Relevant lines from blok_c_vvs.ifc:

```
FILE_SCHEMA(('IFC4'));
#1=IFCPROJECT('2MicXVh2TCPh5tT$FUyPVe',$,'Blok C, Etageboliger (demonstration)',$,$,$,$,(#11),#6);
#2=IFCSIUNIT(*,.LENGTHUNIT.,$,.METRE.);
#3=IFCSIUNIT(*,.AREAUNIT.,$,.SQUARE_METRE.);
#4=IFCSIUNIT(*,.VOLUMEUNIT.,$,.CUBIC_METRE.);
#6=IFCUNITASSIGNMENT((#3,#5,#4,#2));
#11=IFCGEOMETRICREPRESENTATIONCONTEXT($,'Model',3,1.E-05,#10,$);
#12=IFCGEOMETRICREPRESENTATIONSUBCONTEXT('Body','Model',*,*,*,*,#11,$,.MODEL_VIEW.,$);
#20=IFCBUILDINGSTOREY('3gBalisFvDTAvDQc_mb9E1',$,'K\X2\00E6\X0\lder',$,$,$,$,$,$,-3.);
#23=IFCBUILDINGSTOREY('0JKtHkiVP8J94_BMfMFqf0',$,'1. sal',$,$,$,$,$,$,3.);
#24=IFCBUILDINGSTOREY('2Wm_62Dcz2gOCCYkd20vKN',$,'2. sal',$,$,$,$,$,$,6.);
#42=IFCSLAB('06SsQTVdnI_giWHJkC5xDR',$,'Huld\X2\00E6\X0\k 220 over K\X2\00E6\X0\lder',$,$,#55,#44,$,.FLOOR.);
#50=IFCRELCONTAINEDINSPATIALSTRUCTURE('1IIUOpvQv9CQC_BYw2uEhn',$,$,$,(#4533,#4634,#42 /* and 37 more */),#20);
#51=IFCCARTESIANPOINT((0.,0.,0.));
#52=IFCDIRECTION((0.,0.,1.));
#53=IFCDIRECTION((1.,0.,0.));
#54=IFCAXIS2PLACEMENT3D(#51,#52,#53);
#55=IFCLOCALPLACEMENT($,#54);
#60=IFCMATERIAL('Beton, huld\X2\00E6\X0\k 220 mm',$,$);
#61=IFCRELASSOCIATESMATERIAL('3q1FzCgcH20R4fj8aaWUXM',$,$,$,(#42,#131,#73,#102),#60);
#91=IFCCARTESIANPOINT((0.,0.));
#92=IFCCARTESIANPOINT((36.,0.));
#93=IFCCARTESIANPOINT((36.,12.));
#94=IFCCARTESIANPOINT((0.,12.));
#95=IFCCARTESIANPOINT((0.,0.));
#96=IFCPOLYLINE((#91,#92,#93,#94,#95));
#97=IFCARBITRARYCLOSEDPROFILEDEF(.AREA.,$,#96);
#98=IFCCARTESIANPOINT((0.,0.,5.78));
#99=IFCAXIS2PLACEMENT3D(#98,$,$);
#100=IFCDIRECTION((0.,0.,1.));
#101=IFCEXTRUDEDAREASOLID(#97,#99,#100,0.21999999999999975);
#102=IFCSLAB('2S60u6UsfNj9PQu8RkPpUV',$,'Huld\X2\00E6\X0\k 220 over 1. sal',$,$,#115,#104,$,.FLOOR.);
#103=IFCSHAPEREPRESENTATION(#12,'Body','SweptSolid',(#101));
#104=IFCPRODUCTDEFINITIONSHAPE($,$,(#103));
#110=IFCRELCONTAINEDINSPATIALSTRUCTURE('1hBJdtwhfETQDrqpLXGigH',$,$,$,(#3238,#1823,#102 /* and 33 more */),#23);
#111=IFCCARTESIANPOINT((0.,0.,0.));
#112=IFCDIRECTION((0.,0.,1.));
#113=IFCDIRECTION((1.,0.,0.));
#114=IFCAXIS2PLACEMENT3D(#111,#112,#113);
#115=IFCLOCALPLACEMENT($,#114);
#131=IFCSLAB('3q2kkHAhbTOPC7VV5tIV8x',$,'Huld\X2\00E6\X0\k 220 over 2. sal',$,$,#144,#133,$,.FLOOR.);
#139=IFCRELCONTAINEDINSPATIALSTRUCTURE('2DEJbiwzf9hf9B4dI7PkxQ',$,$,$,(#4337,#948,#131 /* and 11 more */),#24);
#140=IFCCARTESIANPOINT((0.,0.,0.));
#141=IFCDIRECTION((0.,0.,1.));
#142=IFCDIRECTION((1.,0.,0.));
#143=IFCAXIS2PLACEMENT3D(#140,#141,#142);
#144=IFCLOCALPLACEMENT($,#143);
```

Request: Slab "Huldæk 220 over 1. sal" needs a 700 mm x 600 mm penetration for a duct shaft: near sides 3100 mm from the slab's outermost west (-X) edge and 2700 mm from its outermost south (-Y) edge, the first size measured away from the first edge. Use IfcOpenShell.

```python
import numpy as np
import ifcopenshell
import ifcopenshell.api.feature
import ifcopenshell.api.geometry
import ifcopenshell.api.root
import ifcopenshell.geom
import ifcopenshell.util.placement
import ifcopenshell.util.representation
import ifcopenshell.util.shape
import ifcopenshell.util.unit

model = ifcopenshell.open("blok_c_vvs.ifc")
unit_scale = ifcopenshell.util.unit.calculate_unit_scale(model)
settings = ifcopenshell.geom.settings()


def volume(element):
    """Net volume in cubic metres, openings subtracted."""
    shape = ifcopenshell.geom.create_shape(settings, element)
    return ifcopenshell.util.shape.get_volume(shape.geometry)


slab = model.by_guid("2S60u6UsfNj9PQu8RkPpUV")
before = volume(slab)

# Extent in the slab's own axes, in metres. The edges named are its -X and -Y sides.
slab_shape = ifcopenshell.geom.create_shape(settings, slab)
vertices = ifcopenshell.util.shape.get_vertices(slab_shape.geometry)
x_min, y_min, bottom = vertices.min(axis=0)
top = vertices[:, 2].max()

opening = ifcopenshell.api.root.create_entity(model, ifc_class="IfcOpeningElement", name="Duct shaft opening", predefined_type="OPENING")
context = ifcopenshell.util.representation.get_context(model, "Model", "Body", "MODEL_VIEW")
width, depth = 0.7, 0.6
outline = [(0.0, 0.0), (width, 0.0), (width, depth), (0.0, depth), (0.0, 0.0)]
# Overshoot both faces by 50 mm so the cut is clean.
shape = ifcopenshell.api.geometry.add_slab_representation(
    model, context=context, depth=top - bottom + 0.1, polyline=outline
)
ifcopenshell.api.geometry.assign_representation(model, product=opening, representation=shape)

matrix = ifcopenshell.util.placement.get_local_placement(slab.ObjectPlacement)
matrix[:, 3] = matrix @ np.append(np.array([x_min + 3.1, y_min + 2.7, bottom - 0.05]) / unit_scale, 1.0)
ifcopenshell.api.geometry.edit_object_placement(model, product=opening, matrix=matrix, is_si=False)
ifcopenshell.api.feature.add_feature(model, feature=opening, element=slab)

after = volume(slab)

print(f"slab volume {before:.3f} -> {after:.3f} m3")

model.write("blok_c_vvs_updated.ifc")
```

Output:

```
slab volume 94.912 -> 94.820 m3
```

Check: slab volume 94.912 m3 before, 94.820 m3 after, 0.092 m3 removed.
